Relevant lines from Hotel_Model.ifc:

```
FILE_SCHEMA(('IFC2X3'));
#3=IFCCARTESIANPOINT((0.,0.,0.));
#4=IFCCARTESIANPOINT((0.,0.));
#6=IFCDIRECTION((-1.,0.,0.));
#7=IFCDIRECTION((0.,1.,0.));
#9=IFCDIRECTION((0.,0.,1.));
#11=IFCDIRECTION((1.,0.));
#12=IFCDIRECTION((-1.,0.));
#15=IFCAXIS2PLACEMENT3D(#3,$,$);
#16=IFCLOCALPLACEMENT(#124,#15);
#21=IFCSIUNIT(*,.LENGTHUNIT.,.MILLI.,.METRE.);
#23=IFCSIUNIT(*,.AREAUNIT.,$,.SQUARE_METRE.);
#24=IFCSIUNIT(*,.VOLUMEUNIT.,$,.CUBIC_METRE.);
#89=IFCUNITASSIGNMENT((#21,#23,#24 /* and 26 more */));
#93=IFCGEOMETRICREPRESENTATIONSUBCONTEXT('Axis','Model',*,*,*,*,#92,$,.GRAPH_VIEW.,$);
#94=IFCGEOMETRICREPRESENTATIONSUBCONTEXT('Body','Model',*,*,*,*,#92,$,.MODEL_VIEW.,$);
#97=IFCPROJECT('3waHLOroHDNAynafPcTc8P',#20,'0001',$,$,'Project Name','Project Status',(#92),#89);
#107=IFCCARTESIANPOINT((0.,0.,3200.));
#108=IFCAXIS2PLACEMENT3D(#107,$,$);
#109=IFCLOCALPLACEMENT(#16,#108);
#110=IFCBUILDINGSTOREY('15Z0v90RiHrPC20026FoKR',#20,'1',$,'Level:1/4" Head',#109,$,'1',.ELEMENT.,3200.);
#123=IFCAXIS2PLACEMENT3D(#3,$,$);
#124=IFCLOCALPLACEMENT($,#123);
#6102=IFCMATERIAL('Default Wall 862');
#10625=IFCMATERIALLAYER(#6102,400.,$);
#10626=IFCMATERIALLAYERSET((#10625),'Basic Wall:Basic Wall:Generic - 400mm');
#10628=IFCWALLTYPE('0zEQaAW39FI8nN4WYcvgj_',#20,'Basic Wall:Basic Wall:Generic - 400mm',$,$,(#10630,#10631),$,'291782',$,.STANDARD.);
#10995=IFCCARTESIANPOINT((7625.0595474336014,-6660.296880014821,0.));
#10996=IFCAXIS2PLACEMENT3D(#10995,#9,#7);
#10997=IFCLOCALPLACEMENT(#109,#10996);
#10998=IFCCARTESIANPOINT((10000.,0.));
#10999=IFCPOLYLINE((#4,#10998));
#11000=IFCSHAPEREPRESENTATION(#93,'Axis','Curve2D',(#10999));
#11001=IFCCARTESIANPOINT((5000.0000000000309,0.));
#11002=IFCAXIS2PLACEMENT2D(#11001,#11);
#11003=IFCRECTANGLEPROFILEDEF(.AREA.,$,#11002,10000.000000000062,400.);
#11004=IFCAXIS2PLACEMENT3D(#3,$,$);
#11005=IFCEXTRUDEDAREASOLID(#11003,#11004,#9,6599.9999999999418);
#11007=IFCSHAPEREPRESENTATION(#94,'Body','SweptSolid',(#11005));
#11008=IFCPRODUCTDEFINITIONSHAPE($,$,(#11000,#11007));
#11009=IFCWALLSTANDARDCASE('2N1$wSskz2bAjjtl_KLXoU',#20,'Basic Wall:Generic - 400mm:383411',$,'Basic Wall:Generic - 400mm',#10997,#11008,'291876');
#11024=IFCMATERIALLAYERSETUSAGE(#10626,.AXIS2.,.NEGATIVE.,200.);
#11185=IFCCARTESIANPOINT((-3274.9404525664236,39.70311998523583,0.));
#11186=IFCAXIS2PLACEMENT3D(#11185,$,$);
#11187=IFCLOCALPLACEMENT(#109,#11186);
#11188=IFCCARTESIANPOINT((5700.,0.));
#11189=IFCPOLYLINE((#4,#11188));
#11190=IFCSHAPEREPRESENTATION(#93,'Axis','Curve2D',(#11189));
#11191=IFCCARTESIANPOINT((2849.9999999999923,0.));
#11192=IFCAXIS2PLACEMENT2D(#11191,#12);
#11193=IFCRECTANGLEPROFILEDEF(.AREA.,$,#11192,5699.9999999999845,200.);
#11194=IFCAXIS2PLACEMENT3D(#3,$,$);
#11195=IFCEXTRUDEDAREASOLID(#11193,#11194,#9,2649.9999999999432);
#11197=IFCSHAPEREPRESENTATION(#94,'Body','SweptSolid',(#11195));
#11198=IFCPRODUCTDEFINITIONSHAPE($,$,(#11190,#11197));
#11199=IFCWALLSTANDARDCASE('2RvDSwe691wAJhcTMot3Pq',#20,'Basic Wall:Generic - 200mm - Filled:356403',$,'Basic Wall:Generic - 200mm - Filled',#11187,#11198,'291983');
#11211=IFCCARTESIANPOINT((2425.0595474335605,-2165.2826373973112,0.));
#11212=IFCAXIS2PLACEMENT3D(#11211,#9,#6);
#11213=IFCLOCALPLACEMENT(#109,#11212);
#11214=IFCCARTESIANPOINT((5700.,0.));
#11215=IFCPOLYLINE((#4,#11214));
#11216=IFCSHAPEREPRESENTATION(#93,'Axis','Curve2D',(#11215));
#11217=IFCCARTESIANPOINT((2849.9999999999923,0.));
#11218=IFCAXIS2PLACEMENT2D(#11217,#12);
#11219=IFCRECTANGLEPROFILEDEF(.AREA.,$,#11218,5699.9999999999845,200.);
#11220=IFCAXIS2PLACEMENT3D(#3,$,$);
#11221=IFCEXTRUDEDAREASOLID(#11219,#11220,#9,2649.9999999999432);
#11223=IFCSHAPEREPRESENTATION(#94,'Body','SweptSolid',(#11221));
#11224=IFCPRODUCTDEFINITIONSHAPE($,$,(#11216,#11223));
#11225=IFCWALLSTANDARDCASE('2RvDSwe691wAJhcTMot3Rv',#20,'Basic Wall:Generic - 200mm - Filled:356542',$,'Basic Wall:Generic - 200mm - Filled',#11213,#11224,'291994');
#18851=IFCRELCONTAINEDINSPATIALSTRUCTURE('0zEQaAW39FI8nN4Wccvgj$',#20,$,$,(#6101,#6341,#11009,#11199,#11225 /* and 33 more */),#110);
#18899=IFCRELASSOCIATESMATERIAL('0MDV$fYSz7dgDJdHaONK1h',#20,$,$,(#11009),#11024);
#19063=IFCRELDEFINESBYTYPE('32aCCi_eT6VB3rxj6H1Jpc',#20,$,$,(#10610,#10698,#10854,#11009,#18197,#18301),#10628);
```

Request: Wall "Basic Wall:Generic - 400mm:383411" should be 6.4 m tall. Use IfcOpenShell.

```python
import ifcopenshell
import ifcopenshell.geom
import ifcopenshell.util.representation
import ifcopenshell.util.shape
import ifcopenshell.util.unit

model = ifcopenshell.open("Hotel_Model.ifc")
unit_scale = ifcopenshell.util.unit.calculate_unit_scale(model)
settings = ifcopenshell.geom.settings()


def volume(element):
    """Net volume in cubic metres, openings subtracted."""
    shape = ifcopenshell.geom.create_shape(settings, element)
    return ifcopenshell.util.shape.get_volume(shape.geometry)


wall = model.by_id(11009)
before = volume(wall)

body = ifcopenshell.util.representation.get_representation(wall, "Model", "Body")
solid = body.Items[0]
old_height = solid.Depth
solid.Depth = 6.4 / unit_scale
after = volume(wall)

print(f"height {old_height:g} -> {solid.Depth:g}, volume {before:.3f} -> {after:.3f} m3")

model.write("Hotel_Model-out.ifc")
```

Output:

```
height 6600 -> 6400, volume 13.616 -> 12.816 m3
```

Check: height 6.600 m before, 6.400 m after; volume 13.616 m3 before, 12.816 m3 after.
